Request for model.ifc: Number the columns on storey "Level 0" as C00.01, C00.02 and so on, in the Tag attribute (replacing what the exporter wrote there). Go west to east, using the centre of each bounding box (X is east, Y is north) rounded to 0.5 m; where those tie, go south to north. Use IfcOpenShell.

First a look at what the model holds.

```python
import ifcopenshell
import ifcopenshell.util.element
import ifcopenshell.util.placement

model = ifcopenshell.open("model.ifc")
print(model.schema)
storey = next(s for s in model.by_type("IfcBuildingStorey") if s.Name == "Level 0")
columns = [e for e in ifcopenshell.util.element.get_decomposition(storey) if e.is_a("IfcColumn")]
for e in sorted(columns, key=lambda e: e.id()):
    origin = ifcopenshell.util.placement.get_local_placement(e.ObjectPlacement)[:3, 3]
    print(e.id(), e.Tag, e.Name, origin.round(2) + 0.0, sep=" | ")
```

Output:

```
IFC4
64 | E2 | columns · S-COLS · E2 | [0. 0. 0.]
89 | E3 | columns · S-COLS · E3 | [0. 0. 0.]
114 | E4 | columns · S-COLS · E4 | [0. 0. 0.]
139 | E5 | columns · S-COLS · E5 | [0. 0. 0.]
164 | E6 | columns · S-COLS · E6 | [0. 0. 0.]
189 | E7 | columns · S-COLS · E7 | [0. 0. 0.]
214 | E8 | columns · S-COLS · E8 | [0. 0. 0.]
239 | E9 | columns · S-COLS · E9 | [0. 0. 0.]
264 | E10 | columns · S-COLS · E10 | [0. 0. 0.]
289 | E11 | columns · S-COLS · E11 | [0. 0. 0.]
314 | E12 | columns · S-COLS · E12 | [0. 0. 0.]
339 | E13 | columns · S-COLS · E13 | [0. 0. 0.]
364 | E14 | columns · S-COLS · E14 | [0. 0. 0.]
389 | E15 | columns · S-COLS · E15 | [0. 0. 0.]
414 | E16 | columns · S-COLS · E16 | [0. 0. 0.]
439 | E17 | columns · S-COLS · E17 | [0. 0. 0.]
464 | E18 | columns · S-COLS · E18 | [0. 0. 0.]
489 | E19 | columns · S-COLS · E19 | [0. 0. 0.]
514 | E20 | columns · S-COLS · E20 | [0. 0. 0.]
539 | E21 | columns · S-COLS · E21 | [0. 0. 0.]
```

```python
import ifcopenshell
import ifcopenshell.geom
import ifcopenshell.util.element
import ifcopenshell.util.shape

model = ifcopenshell.open("model.ifc")
settings = ifcopenshell.geom.settings()
settings.set("use-world-coords", True)


def centre(element):
    shape = ifcopenshell.geom.create_shape(settings, element)
    return ifcopenshell.util.shape.get_bbox_centroid(shape.geometry)


storey = next(s for s in model.by_type("IfcBuildingStorey") if s.Name == "Level 0")
columns = [e for e in ifcopenshell.util.element.get_decomposition(storey) if e.is_a("IfcColumn")]

# Insertion points can sit at a corner or the storey origin, so sort by the geometry (in metres).
centres = {e: centre(e) for e in columns}
columns.sort(key=lambda e: (round(centres[e][0] / 0.5), centres[e][1]))

for i, e in enumerate(columns, start=1):
    number = f"C00.{i:02d}"
    e.Tag = number
    print(e.id(), number)

model.write("model_v2.ifc")
```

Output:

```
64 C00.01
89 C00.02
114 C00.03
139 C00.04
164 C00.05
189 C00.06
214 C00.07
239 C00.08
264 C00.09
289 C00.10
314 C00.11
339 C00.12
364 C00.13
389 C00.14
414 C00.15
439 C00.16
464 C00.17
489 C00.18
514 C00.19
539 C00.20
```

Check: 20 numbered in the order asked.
